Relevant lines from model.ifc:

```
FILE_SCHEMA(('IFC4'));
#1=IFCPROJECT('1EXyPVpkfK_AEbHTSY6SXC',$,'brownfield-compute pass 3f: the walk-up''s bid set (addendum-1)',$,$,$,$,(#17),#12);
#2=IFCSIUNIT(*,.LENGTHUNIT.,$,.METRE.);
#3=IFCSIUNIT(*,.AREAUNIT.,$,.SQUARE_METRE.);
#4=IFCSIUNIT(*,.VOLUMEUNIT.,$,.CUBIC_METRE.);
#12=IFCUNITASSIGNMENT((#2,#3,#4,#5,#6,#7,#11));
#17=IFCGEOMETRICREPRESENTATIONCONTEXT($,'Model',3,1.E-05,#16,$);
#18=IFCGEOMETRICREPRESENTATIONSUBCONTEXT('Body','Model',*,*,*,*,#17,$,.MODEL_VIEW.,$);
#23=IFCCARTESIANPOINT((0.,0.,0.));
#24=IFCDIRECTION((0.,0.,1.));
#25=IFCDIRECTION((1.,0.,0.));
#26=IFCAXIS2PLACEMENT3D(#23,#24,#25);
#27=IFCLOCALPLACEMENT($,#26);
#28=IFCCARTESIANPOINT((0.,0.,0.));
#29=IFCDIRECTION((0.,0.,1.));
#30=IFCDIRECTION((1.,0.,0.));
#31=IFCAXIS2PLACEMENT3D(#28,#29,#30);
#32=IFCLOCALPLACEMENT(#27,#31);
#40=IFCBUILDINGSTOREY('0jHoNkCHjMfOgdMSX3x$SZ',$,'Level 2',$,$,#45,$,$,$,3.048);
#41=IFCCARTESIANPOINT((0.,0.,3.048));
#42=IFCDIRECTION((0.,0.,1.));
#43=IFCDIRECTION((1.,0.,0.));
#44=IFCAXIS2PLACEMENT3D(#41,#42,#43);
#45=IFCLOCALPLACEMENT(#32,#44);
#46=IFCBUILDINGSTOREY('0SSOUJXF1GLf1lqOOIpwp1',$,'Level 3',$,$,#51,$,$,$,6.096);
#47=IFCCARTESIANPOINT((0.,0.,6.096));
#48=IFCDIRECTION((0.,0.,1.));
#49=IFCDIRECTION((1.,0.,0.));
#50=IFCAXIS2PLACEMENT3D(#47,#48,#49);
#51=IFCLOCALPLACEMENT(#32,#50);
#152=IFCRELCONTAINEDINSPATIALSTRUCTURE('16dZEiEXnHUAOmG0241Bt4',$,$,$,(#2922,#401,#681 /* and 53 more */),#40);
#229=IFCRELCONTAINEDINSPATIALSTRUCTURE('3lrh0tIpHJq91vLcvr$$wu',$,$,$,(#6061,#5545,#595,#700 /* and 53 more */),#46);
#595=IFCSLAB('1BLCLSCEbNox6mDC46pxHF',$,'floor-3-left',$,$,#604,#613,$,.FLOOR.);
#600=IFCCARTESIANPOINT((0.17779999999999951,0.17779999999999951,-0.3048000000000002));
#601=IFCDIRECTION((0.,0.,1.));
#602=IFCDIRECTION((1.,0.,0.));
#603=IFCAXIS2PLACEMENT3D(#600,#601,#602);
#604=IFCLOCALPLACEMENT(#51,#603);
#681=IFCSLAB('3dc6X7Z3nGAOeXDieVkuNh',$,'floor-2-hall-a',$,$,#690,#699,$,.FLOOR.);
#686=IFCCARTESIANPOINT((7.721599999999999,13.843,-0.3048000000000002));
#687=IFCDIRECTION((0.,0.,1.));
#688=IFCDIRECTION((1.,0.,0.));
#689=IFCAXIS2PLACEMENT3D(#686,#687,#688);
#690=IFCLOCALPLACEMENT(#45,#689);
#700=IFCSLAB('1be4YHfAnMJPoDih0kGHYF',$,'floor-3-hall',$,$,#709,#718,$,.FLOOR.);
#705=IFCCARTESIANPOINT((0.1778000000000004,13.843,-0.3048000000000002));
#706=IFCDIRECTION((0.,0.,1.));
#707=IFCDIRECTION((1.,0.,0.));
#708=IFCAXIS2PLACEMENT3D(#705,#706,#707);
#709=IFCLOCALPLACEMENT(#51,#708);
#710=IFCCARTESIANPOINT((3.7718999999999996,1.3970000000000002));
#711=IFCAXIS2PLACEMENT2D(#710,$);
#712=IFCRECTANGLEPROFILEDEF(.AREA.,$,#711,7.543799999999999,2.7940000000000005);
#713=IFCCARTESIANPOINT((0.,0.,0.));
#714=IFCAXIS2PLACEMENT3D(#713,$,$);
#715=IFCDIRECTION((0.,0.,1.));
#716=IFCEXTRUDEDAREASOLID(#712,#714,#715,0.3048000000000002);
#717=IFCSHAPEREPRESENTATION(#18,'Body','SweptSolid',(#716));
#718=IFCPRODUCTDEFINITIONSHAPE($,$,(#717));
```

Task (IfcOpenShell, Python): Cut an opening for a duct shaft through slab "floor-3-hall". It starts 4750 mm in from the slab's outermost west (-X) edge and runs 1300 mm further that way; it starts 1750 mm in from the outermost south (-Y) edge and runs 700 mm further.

```python
import numpy as np
import ifcopenshell
import ifcopenshell.api.feature
import ifcopenshell.api.geometry
import ifcopenshell.api.root
import ifcopenshell.geom
import ifcopenshell.util.placement
import ifcopenshell.util.representation
import ifcopenshell.util.shape
import ifcopenshell.util.unit

model = ifcopenshell.open("model.ifc")
unit_scale = ifcopenshell.util.unit.calculate_unit_scale(model)
settings = ifcopenshell.geom.settings()


def volume(element):
    """Net volume in cubic metres, openings subtracted."""
    shape = ifcopenshell.geom.create_shape(settings, element)
    return ifcopenshell.util.shape.get_volume(shape.geometry)


slab = model.by_id(700)
before = volume(slab)

# Extent in the slab's own axes, in metres. The edges named are its -X and -Y sides.
slab_shape = ifcopenshell.geom.create_shape(settings, slab)
vertices = ifcopenshell.util.shape.get_vertices(slab_shape.geometry)
x_min, y_min, bottom = vertices.min(axis=0)
top = vertices[:, 2].max()

opening = ifcopenshell.api.root.create_entity(model, ifc_class="IfcOpeningElement", name="Duct shaft opening", predefined_type="OPENING")
context = ifcopenshell.util.representation.get_context(model, "Model", "Body", "MODEL_VIEW")
width, depth = 1.3, 0.7
outline = [(0.0, 0.0), (width, 0.0), (width, depth), (0.0, depth), (0.0, 0.0)]
# Overshoot both faces by 50 mm so the cut is clean.
shape = ifcopenshell.api.geometry.add_slab_representation(
    model, context=context, depth=top - bottom + 0.1, polyline=outline
)
ifcopenshell.api.geometry.assign_representation(model, product=opening, representation=shape)

matrix = ifcopenshell.util.placement.get_local_placement(slab.ObjectPlacement)
matrix[:, 3] = matrix @ np.append(np.array([x_min + 4.75, y_min + 1.75, bottom - 0.05]) / unit_scale, 1.0)
ifcopenshell.api.geometry.edit_object_placement(model, product=opening, matrix=matrix, is_si=False)
ifcopenshell.api.feature.add_feature(model, feature=opening, element=slab)

after = volume(slab)

print(f"slab volume {before:.3f} -> {after:.3f} m3")

model.write("model_v2.ifc")
```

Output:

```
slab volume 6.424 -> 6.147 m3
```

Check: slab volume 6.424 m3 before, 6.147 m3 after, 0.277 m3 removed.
